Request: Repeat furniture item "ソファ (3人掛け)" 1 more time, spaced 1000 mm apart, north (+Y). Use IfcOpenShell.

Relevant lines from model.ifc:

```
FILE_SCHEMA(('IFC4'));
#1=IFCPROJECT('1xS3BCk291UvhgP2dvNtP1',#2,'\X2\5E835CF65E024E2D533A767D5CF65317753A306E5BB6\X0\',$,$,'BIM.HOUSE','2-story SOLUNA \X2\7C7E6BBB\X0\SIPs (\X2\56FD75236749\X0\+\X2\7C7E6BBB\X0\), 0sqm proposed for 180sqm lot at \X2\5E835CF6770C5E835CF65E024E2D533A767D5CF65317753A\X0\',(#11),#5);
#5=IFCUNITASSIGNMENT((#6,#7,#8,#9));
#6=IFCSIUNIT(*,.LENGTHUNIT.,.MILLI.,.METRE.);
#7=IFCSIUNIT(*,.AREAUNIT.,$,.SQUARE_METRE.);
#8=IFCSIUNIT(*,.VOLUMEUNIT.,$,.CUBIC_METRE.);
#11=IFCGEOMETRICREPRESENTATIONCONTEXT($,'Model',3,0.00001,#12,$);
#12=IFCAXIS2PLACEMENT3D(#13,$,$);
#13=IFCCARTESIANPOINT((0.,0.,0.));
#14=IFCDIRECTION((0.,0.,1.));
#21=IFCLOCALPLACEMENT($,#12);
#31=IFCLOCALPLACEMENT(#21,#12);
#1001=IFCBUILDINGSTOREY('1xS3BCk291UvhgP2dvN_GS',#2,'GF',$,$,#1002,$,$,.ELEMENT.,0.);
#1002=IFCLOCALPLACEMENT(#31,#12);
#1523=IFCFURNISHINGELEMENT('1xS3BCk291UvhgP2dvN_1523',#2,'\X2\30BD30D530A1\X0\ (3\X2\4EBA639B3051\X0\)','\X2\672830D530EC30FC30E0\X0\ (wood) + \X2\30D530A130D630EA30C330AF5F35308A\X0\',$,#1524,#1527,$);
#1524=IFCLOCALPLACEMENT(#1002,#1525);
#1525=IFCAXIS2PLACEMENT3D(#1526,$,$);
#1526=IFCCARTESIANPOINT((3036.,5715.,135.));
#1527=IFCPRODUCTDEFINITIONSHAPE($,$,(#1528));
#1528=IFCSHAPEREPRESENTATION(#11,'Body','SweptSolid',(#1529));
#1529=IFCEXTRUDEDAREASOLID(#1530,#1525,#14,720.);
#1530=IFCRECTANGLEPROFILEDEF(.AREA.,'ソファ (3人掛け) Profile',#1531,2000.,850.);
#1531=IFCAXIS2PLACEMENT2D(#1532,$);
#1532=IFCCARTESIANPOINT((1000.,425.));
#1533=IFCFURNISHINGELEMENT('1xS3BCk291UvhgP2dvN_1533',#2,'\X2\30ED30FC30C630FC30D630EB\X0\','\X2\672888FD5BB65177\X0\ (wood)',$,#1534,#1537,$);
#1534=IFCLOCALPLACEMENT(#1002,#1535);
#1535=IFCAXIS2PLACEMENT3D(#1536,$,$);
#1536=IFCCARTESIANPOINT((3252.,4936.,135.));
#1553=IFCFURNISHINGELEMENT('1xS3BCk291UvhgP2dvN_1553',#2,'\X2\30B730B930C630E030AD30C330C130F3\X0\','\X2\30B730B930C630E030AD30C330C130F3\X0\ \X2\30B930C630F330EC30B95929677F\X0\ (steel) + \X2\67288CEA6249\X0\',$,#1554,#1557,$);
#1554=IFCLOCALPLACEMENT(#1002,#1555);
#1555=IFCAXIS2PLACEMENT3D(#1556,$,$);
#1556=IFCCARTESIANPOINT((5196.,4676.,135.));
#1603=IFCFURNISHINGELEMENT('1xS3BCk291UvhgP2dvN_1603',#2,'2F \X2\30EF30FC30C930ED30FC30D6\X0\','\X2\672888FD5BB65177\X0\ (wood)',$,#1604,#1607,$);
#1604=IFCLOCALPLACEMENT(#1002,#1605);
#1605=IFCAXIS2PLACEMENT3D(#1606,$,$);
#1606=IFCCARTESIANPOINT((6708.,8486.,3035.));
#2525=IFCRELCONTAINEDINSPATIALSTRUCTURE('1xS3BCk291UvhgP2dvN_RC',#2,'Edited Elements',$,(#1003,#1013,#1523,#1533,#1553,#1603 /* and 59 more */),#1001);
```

```python
import numpy as np
import ifcopenshell
import ifcopenshell.api.geometry
import ifcopenshell.api.root
import ifcopenshell.util.element
import ifcopenshell.util.placement
import ifcopenshell.util.unit

model = ifcopenshell.open("model.ifc")
unit_scale = ifcopenshell.util.unit.calculate_unit_scale(model)


def reuse_history(source, copy):
    """copy_class also copies each property set's owner history, people and application; keep the originals."""
    for rel in copy.IsDefinedBy:
        if rel.is_a("IfcRelDefinesByProperties") and (history := rel.RelatingPropertyDefinition.OwnerHistory):
            rel.RelatingPropertyDefinition.OwnerHistory = source.OwnerHistory
            ifcopenshell.util.element.remove_deep2(model, history)


source = model.by_guid("1xS3BCk291UvhgP2dvN_1523")
base = ifcopenshell.util.placement.get_local_placement(source.ObjectPlacement)
step = np.array([0.0, 1.0, 0.0]) * 1 / unit_scale

for i in range(1, 2):
    copy = ifcopenshell.api.root.copy_class(model, product=source)
    copy.Representation = ifcopenshell.util.element.copy_deep(
        model, source.Representation, exclude=["IfcGeometricRepresentationContext", "IfcRepresentationMap"]
    )
    reuse_history(source, copy)
    matrix = base.copy()
    matrix[:3, 3] += i * step
    print("added at", matrix[:3, 3].round(3) + 0.0)
    ifcopenshell.api.geometry.edit_object_placement(model, product=copy, matrix=matrix, is_si=False)

model.write("model_edited.ifc")
```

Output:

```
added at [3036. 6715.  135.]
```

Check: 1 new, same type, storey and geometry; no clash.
